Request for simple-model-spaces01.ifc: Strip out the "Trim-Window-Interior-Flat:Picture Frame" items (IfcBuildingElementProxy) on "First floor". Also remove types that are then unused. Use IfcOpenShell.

First a look at what the model holds.

```python
import ifcopenshell
import ifcopenshell.util.element

model = ifcopenshell.open("simple-model-spaces01.ifc")
print(model.schema)
storey = next(s for s in model.by_type("IfcBuildingStorey") if s.Name == "First floor")
proxies = [e for e in ifcopenshell.util.element.get_decomposition(storey) if e.is_a("IfcBuildingElementProxy")]
seen = {}
for e in proxies:
    element_type = ifcopenshell.util.element.get_type(e)
    name = element_type.Name if element_type not in (None, e) else None
    seen[name] = seen.get(name, 0) + 1
for name, count in sorted(seen.items(), key=str):
    print(count, "x", name)
```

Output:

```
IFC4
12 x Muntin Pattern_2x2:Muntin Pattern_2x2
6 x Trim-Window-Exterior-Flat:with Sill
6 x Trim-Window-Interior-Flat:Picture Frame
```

```python
import ifcopenshell
import ifcopenshell.api.root
import ifcopenshell.util.element

model = ifcopenshell.open("simple-model-spaces01.ifc")

storey = next(s for s in model.by_type("IfcBuildingStorey") if s.Name == "First floor")
proxies = [e for e in ifcopenshell.util.element.get_decomposition(storey) if e.is_a("IfcBuildingElementProxy")]
targets = [e for e in proxies if (t := ifcopenshell.util.element.get_type(e)) not in (None, e) and t.Name == "Trim-Window-Interior-Flat:Picture Frame"]
types = {ifcopenshell.util.element.get_type(e) for e in targets} - {None, *targets}

for e in targets:
    ifcopenshell.api.root.remove_product(model, product=e)
print(len(targets), "removed")

unused = [t for t in types if not ifcopenshell.util.element.get_types(t)]
for t in unused:
    ifcopenshell.api.root.remove_product(model, product=t)
print(len(unused), "unused types removed")

model.write("simple-model-spaces01_edited.ifc")
```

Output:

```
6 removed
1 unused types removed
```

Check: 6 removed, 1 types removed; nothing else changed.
